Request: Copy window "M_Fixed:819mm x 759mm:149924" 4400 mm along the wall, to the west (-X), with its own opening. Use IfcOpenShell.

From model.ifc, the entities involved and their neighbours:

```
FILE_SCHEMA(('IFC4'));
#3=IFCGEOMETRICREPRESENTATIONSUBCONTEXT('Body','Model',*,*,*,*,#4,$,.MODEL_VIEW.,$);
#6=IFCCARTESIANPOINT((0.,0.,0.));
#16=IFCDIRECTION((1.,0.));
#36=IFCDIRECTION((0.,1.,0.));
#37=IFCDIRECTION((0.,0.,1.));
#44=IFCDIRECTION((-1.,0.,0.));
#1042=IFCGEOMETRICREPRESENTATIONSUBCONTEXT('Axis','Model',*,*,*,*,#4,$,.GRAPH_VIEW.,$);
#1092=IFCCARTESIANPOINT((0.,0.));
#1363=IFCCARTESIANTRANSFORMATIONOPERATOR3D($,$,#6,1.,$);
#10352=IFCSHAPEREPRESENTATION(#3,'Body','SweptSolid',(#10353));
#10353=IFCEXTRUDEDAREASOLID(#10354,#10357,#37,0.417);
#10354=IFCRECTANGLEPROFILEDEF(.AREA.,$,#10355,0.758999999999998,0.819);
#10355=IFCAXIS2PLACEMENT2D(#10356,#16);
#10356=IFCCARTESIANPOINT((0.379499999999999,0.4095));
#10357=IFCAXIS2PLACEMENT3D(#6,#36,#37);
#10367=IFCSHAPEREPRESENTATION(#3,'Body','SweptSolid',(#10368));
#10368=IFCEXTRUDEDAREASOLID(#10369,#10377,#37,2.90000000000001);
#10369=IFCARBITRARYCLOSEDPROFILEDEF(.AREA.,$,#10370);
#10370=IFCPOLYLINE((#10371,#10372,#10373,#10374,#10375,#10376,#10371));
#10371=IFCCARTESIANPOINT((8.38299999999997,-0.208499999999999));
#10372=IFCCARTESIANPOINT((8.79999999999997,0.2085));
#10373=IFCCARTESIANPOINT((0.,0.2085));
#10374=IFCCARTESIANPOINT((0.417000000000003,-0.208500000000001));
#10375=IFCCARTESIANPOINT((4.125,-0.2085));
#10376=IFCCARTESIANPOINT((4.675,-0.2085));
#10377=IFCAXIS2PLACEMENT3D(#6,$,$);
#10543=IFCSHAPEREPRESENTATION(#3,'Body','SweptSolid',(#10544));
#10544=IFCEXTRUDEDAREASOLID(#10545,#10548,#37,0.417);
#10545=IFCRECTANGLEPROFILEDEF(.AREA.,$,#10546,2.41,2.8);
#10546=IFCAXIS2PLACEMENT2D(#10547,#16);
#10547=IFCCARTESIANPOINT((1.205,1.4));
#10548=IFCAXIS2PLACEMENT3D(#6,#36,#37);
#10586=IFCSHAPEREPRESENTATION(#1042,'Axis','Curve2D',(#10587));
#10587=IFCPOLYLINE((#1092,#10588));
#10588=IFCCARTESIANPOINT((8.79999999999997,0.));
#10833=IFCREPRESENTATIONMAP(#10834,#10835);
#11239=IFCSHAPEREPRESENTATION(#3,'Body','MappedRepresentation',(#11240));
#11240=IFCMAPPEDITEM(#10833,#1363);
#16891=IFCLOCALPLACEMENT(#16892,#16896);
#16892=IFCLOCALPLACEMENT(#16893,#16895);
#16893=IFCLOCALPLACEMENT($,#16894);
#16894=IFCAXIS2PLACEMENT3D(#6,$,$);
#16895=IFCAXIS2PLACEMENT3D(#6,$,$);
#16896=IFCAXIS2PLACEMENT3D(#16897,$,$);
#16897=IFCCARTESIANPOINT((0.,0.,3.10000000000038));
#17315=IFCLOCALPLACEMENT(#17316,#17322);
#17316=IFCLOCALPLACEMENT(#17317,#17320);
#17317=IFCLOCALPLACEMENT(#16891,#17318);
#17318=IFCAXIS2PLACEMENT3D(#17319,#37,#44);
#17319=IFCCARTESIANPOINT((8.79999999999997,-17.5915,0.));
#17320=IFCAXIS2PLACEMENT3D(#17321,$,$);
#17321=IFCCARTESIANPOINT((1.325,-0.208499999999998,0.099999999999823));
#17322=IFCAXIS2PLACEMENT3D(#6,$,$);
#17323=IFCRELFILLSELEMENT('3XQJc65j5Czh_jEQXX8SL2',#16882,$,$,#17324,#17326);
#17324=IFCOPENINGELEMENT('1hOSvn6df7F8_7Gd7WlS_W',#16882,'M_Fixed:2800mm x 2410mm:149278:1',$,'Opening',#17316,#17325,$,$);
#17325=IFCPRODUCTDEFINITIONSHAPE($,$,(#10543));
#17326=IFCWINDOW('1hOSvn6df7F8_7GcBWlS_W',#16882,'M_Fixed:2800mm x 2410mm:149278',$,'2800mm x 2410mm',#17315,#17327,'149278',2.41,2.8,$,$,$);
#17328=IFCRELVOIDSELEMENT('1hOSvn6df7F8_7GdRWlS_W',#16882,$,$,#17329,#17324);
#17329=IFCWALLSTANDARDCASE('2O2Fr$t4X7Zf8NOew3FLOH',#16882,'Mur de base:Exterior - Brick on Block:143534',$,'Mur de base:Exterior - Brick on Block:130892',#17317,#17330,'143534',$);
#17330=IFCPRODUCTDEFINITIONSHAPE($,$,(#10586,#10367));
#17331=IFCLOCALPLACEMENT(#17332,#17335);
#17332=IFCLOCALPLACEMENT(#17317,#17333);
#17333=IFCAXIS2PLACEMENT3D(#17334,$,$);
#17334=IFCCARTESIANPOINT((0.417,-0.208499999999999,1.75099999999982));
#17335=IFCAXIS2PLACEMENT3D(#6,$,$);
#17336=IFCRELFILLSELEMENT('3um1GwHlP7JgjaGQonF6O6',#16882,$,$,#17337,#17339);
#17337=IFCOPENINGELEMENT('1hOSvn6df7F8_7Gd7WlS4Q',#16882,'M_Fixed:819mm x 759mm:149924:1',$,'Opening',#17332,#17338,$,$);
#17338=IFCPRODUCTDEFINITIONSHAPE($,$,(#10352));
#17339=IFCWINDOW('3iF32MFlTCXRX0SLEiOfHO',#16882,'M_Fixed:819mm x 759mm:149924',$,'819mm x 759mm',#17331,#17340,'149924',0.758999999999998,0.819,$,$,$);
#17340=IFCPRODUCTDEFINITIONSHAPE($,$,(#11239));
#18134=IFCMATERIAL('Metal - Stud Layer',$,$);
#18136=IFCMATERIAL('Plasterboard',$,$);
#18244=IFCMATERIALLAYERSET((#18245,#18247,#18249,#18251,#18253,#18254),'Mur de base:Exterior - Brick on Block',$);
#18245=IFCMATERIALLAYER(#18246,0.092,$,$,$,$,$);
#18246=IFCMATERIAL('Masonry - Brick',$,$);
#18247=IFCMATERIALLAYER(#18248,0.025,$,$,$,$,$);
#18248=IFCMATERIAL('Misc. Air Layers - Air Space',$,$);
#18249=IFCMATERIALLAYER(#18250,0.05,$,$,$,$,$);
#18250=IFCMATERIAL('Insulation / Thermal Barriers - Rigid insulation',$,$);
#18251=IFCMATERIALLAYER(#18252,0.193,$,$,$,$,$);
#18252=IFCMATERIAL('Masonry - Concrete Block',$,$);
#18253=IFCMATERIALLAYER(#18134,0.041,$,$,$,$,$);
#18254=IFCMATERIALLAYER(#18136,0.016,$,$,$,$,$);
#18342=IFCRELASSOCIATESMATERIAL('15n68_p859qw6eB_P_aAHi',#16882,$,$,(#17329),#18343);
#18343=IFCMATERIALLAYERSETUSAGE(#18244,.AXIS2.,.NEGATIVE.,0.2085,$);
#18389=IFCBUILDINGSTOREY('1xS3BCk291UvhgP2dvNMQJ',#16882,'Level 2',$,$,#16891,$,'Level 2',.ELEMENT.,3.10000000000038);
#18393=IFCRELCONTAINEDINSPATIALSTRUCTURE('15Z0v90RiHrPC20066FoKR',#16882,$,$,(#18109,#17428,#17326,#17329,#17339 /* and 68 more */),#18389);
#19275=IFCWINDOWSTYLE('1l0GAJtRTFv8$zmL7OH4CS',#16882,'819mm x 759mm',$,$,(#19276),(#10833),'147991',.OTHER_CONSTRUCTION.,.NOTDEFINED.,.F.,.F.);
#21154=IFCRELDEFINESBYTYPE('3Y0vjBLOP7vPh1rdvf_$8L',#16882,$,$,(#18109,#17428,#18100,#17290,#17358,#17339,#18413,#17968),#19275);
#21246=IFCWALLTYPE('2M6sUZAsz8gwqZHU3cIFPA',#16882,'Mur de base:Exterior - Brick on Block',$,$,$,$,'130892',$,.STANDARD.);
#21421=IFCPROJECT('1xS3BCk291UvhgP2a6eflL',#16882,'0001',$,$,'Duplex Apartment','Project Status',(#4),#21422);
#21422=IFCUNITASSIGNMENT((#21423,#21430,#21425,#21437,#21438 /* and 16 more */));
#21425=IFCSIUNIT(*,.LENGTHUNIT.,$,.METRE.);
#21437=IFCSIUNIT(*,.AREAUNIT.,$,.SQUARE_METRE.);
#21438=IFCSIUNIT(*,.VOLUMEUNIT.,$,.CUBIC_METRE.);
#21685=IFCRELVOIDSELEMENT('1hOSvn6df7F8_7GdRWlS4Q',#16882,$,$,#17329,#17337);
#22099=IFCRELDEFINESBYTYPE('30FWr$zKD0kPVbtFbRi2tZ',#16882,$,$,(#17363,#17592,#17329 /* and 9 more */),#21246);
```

```python
import ifcopenshell
import ifcopenshell.api.feature
import ifcopenshell.api.geometry
import ifcopenshell.api.root
import ifcopenshell.geom
import ifcopenshell.util.element
import ifcopenshell.util.placement
import ifcopenshell.util.shape

model = ifcopenshell.open("model.ifc")
settings = ifcopenshell.geom.settings()


def volume(element):
    """Net volume in cubic metres, openings subtracted."""
    shape = ifcopenshell.geom.create_shape(settings, element)
    return ifcopenshell.util.shape.get_volume(shape.geometry)


def reuse_history(source, copy):
    """copy_class also copies each property set's owner history, people and application; keep the originals."""
    for rel in copy.IsDefinedBy:
        if rel.is_a("IfcRelDefinesByProperties") and (history := rel.RelatingPropertyDefinition.OwnerHistory):
            rel.RelatingPropertyDefinition.OwnerHistory = source.OwnerHistory
            ifcopenshell.util.element.remove_deep2(model, history)


window = model.by_id(17339)
opening = window.FillsVoids[0].RelatingOpeningElement
wall = opening.VoidsElements[0].RelatingBuildingElement
before = volume(wall)
shift = ifcopenshell.util.placement.get_local_placement(wall.ObjectPlacement)[:3, 0] * 4.4

# copy_class copies the void relationship, type, container and properties, but no geometry.
new_opening = ifcopenshell.api.root.copy_class(model, product=opening)
new_opening.Representation = ifcopenshell.util.element.copy_deep(
    model, opening.Representation, exclude=["IfcGeometricRepresentationContext", "IfcRepresentationMap"]
)
new_opening.Name = "M_Fixed:819mm x 759mm"
new_window = ifcopenshell.api.root.copy_class(model, product=window)
new_window.Representation = ifcopenshell.util.element.copy_deep(
    model, window.Representation, exclude=["IfcGeometricRepresentationContext", "IfcRepresentationMap"]
)
new_window.Name = "M_Fixed:819mm x 759mm"
new_window.Tag = None
reuse_history(window, new_window)
ifcopenshell.api.feature.add_filling(model, opening=new_opening, element=new_window)

for old, new in ((opening, new_opening), (window, new_window)):
    matrix = ifcopenshell.util.placement.get_local_placement(old.ObjectPlacement)
    matrix[:3, 3] += shift
    ifcopenshell.api.geometry.edit_object_placement(model, product=new, matrix=matrix, is_si=False)

after = volume(wall)

print(f"wall volume {before:.3f} -> {after:.3f} m3")

model.write("model_v2.ifc")
```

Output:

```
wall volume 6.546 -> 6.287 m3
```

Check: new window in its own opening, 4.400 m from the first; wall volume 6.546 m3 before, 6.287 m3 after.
